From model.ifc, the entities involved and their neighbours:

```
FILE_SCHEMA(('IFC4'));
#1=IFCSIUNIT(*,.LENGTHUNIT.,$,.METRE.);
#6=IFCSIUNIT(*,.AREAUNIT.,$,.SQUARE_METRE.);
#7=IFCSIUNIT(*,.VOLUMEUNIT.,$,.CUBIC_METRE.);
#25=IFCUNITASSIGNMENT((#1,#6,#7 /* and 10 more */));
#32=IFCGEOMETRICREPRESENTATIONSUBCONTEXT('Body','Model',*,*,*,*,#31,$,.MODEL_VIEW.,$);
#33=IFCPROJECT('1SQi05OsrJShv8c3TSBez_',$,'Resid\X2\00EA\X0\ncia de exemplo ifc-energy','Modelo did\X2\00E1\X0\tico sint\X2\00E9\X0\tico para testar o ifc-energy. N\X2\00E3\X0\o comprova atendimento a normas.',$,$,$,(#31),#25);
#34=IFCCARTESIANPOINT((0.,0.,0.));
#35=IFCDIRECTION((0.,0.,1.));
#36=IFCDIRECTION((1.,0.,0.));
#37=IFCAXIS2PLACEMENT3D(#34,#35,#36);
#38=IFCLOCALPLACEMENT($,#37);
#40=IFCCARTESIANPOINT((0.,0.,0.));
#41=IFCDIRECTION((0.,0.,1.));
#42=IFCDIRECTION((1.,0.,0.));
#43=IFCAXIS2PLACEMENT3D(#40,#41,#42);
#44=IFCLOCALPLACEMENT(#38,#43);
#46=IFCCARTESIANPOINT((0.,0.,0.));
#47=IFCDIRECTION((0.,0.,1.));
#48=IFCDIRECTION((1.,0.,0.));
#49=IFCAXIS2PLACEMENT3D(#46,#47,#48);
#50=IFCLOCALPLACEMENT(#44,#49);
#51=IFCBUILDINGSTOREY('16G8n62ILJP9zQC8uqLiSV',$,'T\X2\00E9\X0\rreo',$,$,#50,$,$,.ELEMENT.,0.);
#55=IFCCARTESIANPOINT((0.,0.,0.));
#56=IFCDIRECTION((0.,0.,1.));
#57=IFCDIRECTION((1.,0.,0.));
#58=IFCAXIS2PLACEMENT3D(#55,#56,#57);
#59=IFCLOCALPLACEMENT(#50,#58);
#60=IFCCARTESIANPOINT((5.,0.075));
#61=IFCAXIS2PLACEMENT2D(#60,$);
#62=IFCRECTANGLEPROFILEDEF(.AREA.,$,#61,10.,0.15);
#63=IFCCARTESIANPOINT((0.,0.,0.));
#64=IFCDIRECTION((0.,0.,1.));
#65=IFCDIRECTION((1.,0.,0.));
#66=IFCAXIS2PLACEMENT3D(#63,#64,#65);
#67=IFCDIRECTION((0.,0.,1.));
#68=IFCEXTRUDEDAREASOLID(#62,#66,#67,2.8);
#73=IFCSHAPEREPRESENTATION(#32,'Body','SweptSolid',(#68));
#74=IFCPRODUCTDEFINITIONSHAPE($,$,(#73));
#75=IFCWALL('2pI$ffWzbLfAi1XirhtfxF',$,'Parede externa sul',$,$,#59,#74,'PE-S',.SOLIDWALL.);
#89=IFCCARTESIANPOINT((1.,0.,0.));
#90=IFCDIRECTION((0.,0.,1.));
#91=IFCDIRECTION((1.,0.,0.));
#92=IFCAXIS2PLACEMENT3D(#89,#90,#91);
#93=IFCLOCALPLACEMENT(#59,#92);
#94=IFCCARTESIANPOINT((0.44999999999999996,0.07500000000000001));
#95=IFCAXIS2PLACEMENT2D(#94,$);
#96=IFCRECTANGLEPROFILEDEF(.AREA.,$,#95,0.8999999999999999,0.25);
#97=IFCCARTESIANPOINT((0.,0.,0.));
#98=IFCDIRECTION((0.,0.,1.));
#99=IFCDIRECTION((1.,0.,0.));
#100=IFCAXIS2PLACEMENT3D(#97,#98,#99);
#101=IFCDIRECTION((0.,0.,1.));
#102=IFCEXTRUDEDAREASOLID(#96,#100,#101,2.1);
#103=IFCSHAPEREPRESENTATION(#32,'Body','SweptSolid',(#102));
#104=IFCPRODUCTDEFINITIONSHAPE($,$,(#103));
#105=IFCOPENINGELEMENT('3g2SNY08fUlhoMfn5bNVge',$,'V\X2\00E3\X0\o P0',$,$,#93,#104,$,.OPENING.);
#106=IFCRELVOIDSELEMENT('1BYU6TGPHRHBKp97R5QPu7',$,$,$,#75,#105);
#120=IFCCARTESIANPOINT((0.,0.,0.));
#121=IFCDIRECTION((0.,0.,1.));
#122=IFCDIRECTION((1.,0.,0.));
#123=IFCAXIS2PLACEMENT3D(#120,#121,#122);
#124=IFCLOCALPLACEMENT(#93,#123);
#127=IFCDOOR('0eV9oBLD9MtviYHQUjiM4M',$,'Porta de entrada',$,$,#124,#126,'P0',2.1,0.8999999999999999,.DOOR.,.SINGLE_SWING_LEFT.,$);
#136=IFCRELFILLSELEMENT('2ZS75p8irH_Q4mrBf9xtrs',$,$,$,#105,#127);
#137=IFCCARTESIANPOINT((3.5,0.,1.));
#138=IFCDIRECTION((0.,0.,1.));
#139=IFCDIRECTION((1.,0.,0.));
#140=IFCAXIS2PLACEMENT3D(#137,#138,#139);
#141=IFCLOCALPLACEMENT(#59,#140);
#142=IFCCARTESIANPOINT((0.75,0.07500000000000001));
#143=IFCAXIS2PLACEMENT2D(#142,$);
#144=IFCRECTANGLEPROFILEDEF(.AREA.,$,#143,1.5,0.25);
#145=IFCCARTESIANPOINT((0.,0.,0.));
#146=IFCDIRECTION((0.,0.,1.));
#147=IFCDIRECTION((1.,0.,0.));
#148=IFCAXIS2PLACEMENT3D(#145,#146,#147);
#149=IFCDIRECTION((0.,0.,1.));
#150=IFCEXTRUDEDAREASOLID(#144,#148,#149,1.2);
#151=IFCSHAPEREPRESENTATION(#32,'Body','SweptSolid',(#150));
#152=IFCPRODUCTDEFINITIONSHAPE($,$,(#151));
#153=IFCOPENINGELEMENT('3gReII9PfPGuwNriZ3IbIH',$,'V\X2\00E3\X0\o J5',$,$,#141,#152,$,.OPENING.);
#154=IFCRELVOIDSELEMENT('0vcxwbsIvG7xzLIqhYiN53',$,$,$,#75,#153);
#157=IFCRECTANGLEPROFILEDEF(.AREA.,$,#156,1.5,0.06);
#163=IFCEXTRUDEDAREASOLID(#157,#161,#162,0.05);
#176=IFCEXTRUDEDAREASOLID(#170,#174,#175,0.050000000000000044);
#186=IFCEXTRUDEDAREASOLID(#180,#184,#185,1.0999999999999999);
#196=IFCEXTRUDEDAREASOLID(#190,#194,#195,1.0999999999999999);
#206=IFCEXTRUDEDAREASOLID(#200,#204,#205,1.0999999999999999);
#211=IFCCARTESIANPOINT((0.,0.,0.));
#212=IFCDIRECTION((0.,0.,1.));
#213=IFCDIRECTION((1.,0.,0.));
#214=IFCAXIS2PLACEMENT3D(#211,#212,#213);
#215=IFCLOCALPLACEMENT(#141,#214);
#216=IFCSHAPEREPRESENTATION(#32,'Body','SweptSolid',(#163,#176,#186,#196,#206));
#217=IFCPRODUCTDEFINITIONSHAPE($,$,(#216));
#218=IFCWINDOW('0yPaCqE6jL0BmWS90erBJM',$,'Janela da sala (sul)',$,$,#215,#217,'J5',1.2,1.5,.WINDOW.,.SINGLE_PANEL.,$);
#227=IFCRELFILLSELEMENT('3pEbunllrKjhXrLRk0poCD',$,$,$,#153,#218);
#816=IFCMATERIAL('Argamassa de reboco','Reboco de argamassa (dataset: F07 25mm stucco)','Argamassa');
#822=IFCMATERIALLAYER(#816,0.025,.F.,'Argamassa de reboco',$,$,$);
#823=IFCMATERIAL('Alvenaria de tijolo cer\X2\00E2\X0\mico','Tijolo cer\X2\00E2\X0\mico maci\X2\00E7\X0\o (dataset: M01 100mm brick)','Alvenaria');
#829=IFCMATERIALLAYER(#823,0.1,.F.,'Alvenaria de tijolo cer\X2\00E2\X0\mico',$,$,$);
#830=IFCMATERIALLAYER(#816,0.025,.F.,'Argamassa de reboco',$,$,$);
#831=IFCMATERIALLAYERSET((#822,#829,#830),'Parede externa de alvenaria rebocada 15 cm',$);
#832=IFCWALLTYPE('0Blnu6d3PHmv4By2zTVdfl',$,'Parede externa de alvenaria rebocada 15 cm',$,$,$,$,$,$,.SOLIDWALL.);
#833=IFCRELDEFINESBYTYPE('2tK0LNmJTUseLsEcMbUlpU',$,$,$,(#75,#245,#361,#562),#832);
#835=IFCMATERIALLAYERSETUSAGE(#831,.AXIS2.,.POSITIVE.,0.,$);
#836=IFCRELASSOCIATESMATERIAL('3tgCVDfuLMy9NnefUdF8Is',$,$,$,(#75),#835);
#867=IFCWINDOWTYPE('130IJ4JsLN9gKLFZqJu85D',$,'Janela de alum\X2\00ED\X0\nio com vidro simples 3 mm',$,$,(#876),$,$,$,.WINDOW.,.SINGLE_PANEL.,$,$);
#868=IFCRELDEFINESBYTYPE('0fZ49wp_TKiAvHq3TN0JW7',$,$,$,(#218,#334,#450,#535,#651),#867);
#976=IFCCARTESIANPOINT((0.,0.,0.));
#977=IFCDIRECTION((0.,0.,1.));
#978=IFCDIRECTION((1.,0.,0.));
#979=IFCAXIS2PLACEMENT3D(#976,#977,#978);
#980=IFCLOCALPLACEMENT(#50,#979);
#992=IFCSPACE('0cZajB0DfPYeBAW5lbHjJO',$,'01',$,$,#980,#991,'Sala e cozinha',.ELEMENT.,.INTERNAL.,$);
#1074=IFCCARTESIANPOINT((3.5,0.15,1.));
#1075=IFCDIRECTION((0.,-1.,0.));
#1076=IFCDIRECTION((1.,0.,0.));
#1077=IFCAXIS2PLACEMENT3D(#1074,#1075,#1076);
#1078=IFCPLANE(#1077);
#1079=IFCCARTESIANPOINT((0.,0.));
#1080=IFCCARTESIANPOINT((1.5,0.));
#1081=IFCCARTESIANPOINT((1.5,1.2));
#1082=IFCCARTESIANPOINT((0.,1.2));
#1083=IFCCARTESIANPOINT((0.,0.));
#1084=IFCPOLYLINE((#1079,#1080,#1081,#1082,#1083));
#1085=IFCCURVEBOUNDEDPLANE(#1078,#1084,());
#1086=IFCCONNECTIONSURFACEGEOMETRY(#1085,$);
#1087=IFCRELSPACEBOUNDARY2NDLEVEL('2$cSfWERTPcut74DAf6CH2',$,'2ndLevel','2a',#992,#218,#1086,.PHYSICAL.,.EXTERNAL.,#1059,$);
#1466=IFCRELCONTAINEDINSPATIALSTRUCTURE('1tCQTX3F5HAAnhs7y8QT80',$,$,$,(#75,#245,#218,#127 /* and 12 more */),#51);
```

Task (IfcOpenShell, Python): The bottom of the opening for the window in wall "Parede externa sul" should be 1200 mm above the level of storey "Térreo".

```python
import numpy as np
import ifcopenshell
import ifcopenshell.api.geometry
import ifcopenshell.geom
import ifcopenshell.util.element
import ifcopenshell.util.placement
import ifcopenshell.util.shape
import ifcopenshell.util.unit

model = ifcopenshell.open("model.ifc")
unit_scale = ifcopenshell.util.unit.calculate_unit_scale(model)

window = model.by_id(218)
opening = window.FillsVoids[0].RelatingOpeningElement
storey = ifcopenshell.util.element.get_container(window, ifc_class="IfcBuildingStorey")
level = ifcopenshell.util.placement.get_local_placement(storey.ObjectPlacement)[2, 3]

# The opening's origin need not be at the sill, so measure its lowest point.
shape = ifcopenshell.geom.create_shape(ifcopenshell.geom.settings(), opening)
bottom = ifcopenshell.util.shape.get_shape_bottom_elevation(shape, shape.geometry) / unit_scale
dz = level + 1.2 - bottom

shift = np.array([0.0, 0.0, dz])
# The window is placed relative to its opening, so it follows when the opening moves.
matrix = ifcopenshell.util.placement.get_local_placement(opening.ObjectPlacement)
matrix[:3, 3] += shift
ifcopenshell.api.geometry.edit_object_placement(
    model, product=opening, matrix=matrix, is_si=False, should_transform_children=True
)

# Space boundary surfaces are stored in each space's coordinates; move them too.
for rel in window.ProvidesBoundaries:
    if not rel.ConnectionGeometry:
        continue
    surface = rel.ConnectionGeometry.SurfaceOnRelatingElement.BasisSurface
    space_matrix = ifcopenshell.util.placement.get_local_placement(rel.RelatingSpace.ObjectPlacement)
    point = np.array(surface.Position.Location.Coordinates) + space_matrix[:3, :3].T @ shift
    surface.Position = model.createIfcAxis2Placement3D(
        model.createIfcCartesianPoint(point.tolist()), surface.Position.Axis, surface.Position.RefDirection
    )

print(f"moved by {dz * unit_scale:+.3f} m")

model.write("model_edited.ifc")
```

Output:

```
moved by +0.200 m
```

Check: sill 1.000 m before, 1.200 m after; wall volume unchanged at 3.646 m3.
